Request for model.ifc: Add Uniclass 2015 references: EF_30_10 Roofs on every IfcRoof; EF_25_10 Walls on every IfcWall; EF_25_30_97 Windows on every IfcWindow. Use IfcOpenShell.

First a look at what the model holds.

```python
import ifcopenshell

model = ifcopenshell.open("model.ifc")
print(model.schema)
print("classifications:", [c.Name for c in model.by_type("IfcClassification")])
for ifc_class in ("IfcDoor", "IfcRoof", "IfcStair", "IfcWall", "IfcWindow"):
    print(ifc_class, len(model.by_type(ifc_class)))
```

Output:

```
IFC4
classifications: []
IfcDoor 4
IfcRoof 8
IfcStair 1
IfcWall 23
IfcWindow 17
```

```python
import ifcopenshell
import ifcopenshell.api.classification

model = ifcopenshell.open("model.ifc")

system = ifcopenshell.api.classification.add_classification(model, classification="Uniclass 2015")

codes = {
    "IfcRoof": ("EF_30_10", "Roofs"),
    "IfcWall": ("EF_25_10", "Walls"),
    "IfcWindow": ("EF_25_30_97", "Windows"),
}
for ifc_class, (code, name) in codes.items():
    products = model.by_type(ifc_class)
    ifcopenshell.api.classification.add_reference(
        model, products=products, classification=system, identification=code, name=name
    )
    print(code, len(products))

model.write("model_edited.ifc")
```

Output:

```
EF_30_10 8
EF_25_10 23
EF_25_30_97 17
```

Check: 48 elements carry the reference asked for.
